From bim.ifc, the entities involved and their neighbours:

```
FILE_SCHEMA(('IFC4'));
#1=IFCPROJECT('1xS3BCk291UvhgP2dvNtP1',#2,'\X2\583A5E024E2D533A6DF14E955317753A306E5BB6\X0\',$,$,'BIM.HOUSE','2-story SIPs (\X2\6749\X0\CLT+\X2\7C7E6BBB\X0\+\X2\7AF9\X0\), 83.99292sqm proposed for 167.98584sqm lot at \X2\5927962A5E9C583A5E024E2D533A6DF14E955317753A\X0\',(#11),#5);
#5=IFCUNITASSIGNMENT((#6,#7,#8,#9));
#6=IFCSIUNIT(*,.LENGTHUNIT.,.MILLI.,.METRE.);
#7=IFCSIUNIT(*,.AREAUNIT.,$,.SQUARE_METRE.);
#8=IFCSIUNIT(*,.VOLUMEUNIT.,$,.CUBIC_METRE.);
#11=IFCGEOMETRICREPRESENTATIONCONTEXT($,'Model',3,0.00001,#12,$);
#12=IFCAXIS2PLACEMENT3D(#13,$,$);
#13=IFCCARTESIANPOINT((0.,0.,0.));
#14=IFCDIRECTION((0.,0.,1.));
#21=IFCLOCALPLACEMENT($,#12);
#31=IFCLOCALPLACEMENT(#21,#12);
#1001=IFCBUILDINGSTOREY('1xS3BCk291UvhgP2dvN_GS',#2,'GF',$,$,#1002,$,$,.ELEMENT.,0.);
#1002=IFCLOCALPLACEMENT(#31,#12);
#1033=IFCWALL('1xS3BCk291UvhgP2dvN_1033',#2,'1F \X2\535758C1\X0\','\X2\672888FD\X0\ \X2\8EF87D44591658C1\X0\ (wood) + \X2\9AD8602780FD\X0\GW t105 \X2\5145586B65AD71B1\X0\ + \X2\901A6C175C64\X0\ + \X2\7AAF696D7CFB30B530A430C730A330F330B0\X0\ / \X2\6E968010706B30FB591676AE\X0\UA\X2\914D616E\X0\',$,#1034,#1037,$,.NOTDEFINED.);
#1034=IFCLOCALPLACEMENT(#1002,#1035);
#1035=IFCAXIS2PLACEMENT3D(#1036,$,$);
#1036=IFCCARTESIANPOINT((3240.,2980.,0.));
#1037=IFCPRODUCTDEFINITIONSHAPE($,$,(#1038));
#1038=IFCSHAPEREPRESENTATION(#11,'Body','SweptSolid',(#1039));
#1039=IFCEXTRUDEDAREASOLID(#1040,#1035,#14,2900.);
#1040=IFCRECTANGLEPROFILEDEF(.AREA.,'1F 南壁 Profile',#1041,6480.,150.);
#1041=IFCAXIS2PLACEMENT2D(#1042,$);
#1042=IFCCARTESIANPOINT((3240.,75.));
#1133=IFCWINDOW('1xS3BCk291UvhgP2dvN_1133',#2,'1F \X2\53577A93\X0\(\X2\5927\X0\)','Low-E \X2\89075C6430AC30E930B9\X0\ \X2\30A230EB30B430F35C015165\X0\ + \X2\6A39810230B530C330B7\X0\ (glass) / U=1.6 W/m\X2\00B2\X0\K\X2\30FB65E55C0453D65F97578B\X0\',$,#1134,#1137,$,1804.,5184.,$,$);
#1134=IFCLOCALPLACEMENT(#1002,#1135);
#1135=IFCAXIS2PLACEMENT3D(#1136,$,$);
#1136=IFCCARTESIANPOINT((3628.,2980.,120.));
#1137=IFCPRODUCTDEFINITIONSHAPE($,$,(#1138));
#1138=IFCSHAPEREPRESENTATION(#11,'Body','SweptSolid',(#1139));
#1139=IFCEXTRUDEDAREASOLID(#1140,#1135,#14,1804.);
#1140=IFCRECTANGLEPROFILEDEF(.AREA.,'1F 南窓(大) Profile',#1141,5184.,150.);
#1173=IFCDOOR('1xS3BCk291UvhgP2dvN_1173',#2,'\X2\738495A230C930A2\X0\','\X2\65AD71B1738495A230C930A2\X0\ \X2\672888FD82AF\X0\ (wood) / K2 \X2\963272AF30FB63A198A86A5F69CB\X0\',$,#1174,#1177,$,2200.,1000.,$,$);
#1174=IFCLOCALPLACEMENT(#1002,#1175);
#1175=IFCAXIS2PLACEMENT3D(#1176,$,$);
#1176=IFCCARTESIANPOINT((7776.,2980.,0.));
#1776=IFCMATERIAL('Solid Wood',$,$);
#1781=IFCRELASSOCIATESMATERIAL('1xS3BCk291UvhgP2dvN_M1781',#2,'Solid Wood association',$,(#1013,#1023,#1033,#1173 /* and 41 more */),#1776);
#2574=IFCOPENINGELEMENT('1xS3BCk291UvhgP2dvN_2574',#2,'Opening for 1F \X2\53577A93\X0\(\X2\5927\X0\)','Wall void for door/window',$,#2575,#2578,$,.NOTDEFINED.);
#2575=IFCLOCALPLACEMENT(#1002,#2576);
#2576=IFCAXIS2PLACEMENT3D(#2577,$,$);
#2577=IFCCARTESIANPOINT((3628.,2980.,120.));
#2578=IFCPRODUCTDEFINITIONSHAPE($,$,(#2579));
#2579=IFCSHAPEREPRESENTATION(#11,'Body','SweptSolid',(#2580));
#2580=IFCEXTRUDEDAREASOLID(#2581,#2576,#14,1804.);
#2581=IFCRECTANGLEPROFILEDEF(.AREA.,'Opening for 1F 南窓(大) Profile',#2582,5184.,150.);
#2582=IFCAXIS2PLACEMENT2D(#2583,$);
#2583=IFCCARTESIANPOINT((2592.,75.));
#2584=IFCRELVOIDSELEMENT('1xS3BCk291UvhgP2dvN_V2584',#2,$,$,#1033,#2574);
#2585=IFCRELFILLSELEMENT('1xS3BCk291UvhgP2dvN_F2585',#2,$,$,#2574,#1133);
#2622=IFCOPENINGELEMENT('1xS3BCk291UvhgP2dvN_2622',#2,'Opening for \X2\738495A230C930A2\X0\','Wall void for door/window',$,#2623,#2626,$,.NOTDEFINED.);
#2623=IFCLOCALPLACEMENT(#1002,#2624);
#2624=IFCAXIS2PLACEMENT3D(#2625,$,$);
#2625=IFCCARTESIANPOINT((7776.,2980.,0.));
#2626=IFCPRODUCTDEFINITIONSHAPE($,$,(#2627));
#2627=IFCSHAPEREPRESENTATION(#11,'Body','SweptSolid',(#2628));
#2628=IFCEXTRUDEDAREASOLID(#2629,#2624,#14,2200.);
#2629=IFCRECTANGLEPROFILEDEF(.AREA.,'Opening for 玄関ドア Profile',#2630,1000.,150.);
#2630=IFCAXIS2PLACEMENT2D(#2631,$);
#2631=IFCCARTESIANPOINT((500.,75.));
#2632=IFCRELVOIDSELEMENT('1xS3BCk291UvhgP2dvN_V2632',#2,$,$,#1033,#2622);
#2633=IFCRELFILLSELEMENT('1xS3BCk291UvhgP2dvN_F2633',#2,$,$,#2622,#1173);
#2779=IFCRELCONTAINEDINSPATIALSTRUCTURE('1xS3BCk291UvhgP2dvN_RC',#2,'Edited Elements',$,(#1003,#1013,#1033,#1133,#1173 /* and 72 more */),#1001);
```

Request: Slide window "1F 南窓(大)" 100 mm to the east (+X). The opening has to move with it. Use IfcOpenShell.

```python
import ifcopenshell
import ifcopenshell.api.geometry
import ifcopenshell.util.placement
import ifcopenshell.util.unit

model = ifcopenshell.open("bim.ifc")
unit_scale = ifcopenshell.util.unit.calculate_unit_scale(model)

window = model.by_id(1133)
opening = window.FillsVoids[0].RelatingOpeningElement
wall = opening.VoidsElements[0].RelatingBuildingElement

wall_matrix = ifcopenshell.util.placement.get_local_placement(wall.ObjectPlacement)
shift = wall_matrix[:3, 0] * 0.1 / unit_scale
before = ifcopenshell.util.placement.get_local_placement(window.ObjectPlacement)[:3, 3].copy()

# The window is not placed relative to its opening, so move both.
for product in (opening, window):
    matrix = ifcopenshell.util.placement.get_local_placement(product.ObjectPlacement)
    matrix[:3, 3] += shift
    ifcopenshell.api.geometry.edit_object_placement(model, product=product, matrix=matrix, is_si=False)

after = ifcopenshell.util.placement.get_local_placement(window.ObjectPlacement)[:3, 3]
print("window moved by", (after - before).round(3) + 0.0)

model.write("bim_v2.ifc")
```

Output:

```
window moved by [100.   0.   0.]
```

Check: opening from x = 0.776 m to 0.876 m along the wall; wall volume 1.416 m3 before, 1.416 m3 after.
